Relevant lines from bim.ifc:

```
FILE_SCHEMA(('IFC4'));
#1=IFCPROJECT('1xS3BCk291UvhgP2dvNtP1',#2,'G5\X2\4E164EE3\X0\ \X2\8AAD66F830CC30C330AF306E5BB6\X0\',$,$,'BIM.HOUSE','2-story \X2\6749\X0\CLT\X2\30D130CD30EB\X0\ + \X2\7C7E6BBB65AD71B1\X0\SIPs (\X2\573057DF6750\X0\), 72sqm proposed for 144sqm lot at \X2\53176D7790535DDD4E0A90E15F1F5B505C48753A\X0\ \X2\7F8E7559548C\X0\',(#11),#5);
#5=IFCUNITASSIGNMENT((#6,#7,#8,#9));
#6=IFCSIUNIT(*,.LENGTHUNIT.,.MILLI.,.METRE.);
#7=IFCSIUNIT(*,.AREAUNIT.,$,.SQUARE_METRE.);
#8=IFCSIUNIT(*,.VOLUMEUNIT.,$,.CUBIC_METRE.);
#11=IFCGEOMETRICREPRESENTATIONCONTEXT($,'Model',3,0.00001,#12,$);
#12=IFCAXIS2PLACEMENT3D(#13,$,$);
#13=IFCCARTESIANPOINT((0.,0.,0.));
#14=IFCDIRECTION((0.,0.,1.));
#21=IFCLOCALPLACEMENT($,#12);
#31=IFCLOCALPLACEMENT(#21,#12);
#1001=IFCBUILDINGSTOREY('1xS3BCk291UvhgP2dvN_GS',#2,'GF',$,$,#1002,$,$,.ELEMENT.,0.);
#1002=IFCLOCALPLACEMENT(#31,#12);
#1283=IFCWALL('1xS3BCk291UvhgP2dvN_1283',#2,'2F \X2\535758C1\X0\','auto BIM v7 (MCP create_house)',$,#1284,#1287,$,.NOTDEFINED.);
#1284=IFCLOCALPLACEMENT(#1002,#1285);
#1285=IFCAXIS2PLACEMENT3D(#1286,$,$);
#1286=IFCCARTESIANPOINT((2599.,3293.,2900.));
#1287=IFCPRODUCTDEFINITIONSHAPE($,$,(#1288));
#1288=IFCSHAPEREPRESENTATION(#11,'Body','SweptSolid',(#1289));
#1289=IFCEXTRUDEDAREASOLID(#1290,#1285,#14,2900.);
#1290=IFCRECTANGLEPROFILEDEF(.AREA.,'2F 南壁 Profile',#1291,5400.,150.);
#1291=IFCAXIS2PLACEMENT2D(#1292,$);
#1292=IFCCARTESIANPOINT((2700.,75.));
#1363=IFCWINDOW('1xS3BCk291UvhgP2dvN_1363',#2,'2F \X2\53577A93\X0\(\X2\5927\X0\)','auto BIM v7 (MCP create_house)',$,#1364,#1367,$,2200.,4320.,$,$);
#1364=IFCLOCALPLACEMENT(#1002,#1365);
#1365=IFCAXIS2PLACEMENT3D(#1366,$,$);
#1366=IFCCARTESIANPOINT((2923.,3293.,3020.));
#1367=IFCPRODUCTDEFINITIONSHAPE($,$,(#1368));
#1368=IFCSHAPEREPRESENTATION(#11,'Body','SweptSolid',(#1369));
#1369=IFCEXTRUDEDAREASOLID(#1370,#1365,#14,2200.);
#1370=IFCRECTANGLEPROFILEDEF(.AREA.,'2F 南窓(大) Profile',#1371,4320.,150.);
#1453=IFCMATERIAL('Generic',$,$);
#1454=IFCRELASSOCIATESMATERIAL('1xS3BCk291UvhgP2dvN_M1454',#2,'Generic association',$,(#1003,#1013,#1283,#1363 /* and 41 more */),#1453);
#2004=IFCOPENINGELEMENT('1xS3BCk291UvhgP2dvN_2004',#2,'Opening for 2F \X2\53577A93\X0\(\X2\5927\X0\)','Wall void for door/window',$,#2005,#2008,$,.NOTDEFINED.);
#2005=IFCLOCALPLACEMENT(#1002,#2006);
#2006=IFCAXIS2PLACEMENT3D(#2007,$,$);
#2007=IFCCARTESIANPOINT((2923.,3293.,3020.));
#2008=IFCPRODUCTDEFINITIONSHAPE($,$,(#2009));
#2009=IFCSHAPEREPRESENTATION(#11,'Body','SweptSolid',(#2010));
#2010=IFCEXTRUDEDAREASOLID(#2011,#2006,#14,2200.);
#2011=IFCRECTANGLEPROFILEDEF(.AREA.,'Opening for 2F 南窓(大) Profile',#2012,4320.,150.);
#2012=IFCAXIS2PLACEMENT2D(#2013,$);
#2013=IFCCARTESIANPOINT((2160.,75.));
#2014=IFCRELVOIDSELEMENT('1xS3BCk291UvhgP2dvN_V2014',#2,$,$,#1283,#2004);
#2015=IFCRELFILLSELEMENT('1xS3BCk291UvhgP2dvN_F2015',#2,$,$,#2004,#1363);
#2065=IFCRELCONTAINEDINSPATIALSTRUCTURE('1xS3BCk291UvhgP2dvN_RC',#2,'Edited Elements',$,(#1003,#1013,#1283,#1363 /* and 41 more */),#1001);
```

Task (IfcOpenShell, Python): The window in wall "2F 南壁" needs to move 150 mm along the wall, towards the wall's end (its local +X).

```python
import ifcopenshell
import ifcopenshell.api.geometry
import ifcopenshell.util.placement
import ifcopenshell.util.unit

model = ifcopenshell.open("bim.ifc")
unit_scale = ifcopenshell.util.unit.calculate_unit_scale(model)

window = model.by_guid("1xS3BCk291UvhgP2dvN_1363")
opening = window.FillsVoids[0].RelatingOpeningElement
wall = opening.VoidsElements[0].RelatingBuildingElement

wall_matrix = ifcopenshell.util.placement.get_local_placement(wall.ObjectPlacement)
shift = wall_matrix[:3, 0] * 0.15 / unit_scale
before = ifcopenshell.util.placement.get_local_placement(window.ObjectPlacement)[:3, 3].copy()

# The window is not placed relative to its opening, so move both.
for product in (opening, window):
    matrix = ifcopenshell.util.placement.get_local_placement(product.ObjectPlacement)
    matrix[:3, 3] += shift
    ifcopenshell.api.geometry.edit_object_placement(model, product=product, matrix=matrix, is_si=False)

after = ifcopenshell.util.placement.get_local_placement(window.ObjectPlacement)[:3, 3]
print("window moved by", (after - before).round(3) + 0.0)

model.write("bim_rev.ifc")
```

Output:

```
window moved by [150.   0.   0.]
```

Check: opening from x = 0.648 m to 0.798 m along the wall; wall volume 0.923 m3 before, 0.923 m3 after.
